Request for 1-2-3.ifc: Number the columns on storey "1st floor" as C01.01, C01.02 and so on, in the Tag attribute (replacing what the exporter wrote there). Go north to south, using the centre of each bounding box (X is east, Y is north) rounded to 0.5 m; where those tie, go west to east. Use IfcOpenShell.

First a look at what the model holds.

```python
import ifcopenshell
import ifcopenshell.util.element
import ifcopenshell.util.placement

model = ifcopenshell.open("1-2-3.ifc")
print(model.schema)
storey = next(s for s in model.by_type("IfcBuildingStorey") if s.Name == "1st floor")
columns = [e for e in ifcopenshell.util.element.get_decomposition(storey) if e.is_a("IfcColumn")]
for e in sorted(columns, key=lambda e: e.id()):
    origin = ifcopenshell.util.placement.get_local_placement(e.ObjectPlacement)[:3, 3]
    print(e.id(), e.Tag, e.Name, origin.round(2) + 0.0, sep=" | ")
```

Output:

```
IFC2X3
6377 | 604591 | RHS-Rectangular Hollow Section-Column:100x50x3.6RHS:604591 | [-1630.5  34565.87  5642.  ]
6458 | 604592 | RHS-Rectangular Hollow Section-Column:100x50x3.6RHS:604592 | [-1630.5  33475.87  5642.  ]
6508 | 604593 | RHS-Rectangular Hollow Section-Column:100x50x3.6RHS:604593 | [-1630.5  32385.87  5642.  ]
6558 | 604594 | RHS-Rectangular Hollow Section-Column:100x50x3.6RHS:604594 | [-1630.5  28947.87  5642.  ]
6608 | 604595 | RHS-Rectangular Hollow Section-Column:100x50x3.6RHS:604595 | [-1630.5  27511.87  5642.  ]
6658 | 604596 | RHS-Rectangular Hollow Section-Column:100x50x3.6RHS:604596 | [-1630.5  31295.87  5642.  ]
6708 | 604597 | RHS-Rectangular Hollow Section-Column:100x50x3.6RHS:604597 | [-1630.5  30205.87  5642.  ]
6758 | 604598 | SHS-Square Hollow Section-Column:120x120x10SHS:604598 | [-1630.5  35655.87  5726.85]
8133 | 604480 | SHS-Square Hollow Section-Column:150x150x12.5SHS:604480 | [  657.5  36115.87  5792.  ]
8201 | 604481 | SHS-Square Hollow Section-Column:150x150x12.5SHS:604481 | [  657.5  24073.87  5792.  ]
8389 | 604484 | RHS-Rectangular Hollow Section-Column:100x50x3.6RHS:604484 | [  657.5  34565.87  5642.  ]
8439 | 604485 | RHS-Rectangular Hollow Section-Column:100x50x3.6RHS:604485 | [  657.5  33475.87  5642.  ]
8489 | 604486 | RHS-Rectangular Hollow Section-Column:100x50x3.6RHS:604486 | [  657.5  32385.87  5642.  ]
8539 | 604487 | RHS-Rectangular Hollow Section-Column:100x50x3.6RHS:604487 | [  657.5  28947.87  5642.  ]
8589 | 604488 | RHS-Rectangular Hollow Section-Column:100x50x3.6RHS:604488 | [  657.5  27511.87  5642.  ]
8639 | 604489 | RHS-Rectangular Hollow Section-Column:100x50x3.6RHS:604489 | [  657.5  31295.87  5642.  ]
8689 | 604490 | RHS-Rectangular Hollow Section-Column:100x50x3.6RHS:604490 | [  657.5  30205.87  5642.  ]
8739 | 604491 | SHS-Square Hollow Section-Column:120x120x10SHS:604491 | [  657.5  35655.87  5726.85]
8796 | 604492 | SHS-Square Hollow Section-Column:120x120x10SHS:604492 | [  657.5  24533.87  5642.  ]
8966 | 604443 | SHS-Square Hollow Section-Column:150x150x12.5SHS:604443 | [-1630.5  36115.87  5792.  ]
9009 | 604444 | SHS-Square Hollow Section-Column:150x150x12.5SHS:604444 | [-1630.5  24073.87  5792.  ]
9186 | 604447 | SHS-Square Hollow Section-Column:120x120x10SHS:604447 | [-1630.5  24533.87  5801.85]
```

```python
import ifcopenshell
import ifcopenshell.geom
import ifcopenshell.util.element
import ifcopenshell.util.shape

model = ifcopenshell.open("1-2-3.ifc")
settings = ifcopenshell.geom.settings()
settings.set("use-world-coords", True)


def centre(element):
    shape = ifcopenshell.geom.create_shape(settings, element)
    return ifcopenshell.util.shape.get_bbox_centroid(shape.geometry)


storey = next(s for s in model.by_type("IfcBuildingStorey") if s.Name == "1st floor")
columns = [e for e in ifcopenshell.util.element.get_decomposition(storey) if e.is_a("IfcColumn")]

# Insertion points can sit at a corner or the storey origin, so sort by the geometry (in metres).
centres = {e: centre(e) for e in columns}
columns.sort(key=lambda e: (-round(centres[e][1] / 0.5), centres[e][0]))

for i, e in enumerate(columns, start=1):
    number = f"C01.{i:02d}"
    e.Tag = number
    print(e.id(), number)

model.write("1-2-3_v2.ifc")
```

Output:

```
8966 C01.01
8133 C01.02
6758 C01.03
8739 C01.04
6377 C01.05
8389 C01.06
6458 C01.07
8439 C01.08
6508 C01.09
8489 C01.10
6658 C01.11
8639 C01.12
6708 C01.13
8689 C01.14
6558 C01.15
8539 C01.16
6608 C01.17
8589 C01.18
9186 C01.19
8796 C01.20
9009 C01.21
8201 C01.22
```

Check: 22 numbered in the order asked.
